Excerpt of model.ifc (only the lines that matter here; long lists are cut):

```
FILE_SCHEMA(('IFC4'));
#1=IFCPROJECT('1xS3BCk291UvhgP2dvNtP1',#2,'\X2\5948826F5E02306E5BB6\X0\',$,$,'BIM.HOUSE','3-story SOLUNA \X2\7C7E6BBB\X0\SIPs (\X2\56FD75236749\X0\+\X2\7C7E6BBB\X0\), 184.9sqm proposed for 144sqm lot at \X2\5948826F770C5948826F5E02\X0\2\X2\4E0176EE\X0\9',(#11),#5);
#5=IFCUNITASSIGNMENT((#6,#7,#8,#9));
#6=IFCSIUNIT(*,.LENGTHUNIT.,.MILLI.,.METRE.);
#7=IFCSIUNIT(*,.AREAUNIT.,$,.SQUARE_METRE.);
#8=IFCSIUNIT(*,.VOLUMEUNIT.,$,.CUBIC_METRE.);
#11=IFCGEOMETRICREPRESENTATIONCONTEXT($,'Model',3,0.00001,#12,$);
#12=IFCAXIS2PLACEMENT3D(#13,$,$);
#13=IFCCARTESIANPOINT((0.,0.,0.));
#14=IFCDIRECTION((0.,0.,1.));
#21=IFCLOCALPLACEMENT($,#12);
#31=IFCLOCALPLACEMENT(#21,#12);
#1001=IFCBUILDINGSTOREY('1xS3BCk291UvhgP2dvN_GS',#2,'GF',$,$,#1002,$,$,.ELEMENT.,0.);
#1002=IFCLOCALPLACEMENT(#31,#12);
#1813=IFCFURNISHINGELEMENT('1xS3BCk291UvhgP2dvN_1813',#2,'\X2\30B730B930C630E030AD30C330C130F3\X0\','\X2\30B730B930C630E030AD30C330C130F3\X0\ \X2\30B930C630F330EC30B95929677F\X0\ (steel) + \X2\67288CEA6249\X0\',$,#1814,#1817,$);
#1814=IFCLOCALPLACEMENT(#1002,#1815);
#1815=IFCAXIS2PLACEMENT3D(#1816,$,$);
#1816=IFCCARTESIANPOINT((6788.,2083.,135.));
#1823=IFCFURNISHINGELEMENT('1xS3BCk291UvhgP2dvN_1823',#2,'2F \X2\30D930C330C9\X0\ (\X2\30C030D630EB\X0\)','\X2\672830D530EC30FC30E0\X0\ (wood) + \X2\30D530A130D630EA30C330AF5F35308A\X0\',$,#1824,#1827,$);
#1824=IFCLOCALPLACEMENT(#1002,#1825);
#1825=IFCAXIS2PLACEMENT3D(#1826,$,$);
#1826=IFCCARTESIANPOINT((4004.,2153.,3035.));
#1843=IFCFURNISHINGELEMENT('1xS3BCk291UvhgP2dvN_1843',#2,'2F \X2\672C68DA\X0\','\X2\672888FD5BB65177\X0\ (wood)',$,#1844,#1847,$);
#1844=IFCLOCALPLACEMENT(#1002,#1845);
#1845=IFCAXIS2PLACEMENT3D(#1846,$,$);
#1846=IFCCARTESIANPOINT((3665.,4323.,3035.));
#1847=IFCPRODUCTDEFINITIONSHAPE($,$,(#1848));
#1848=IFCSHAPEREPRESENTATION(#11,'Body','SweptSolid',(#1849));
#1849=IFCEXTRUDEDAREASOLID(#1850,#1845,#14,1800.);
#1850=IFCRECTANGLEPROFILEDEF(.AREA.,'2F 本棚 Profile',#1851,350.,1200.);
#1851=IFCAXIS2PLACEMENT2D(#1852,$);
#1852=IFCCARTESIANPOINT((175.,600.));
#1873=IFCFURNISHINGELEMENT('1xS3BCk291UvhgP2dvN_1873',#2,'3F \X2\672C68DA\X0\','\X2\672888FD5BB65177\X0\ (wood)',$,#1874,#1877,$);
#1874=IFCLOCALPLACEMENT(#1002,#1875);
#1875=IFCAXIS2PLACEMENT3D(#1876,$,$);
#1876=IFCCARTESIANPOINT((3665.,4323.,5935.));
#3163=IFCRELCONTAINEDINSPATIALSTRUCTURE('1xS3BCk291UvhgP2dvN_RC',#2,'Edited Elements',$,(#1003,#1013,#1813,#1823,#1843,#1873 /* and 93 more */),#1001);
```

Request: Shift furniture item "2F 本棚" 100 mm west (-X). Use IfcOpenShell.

```python
import ifcopenshell
import ifcopenshell.api.geometry
import ifcopenshell.util.placement

model = ifcopenshell.open("model.ifc")

item = model.by_guid("1xS3BCk291UvhgP2dvN_1843")
matrix = ifcopenshell.util.placement.get_local_placement(item.ObjectPlacement)
matrix[0, 3] -= 100.0
ifcopenshell.api.geometry.edit_object_placement(model, product=item, matrix=matrix, is_si=False)

print(ifcopenshell.util.placement.get_local_placement(item.ObjectPlacement).round(3) + 0.0)

model.write("model_rev.ifc")
```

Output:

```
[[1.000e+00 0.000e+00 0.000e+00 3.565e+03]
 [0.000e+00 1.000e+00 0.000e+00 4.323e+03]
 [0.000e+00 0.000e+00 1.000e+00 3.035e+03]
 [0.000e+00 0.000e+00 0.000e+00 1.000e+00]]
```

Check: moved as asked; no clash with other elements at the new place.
